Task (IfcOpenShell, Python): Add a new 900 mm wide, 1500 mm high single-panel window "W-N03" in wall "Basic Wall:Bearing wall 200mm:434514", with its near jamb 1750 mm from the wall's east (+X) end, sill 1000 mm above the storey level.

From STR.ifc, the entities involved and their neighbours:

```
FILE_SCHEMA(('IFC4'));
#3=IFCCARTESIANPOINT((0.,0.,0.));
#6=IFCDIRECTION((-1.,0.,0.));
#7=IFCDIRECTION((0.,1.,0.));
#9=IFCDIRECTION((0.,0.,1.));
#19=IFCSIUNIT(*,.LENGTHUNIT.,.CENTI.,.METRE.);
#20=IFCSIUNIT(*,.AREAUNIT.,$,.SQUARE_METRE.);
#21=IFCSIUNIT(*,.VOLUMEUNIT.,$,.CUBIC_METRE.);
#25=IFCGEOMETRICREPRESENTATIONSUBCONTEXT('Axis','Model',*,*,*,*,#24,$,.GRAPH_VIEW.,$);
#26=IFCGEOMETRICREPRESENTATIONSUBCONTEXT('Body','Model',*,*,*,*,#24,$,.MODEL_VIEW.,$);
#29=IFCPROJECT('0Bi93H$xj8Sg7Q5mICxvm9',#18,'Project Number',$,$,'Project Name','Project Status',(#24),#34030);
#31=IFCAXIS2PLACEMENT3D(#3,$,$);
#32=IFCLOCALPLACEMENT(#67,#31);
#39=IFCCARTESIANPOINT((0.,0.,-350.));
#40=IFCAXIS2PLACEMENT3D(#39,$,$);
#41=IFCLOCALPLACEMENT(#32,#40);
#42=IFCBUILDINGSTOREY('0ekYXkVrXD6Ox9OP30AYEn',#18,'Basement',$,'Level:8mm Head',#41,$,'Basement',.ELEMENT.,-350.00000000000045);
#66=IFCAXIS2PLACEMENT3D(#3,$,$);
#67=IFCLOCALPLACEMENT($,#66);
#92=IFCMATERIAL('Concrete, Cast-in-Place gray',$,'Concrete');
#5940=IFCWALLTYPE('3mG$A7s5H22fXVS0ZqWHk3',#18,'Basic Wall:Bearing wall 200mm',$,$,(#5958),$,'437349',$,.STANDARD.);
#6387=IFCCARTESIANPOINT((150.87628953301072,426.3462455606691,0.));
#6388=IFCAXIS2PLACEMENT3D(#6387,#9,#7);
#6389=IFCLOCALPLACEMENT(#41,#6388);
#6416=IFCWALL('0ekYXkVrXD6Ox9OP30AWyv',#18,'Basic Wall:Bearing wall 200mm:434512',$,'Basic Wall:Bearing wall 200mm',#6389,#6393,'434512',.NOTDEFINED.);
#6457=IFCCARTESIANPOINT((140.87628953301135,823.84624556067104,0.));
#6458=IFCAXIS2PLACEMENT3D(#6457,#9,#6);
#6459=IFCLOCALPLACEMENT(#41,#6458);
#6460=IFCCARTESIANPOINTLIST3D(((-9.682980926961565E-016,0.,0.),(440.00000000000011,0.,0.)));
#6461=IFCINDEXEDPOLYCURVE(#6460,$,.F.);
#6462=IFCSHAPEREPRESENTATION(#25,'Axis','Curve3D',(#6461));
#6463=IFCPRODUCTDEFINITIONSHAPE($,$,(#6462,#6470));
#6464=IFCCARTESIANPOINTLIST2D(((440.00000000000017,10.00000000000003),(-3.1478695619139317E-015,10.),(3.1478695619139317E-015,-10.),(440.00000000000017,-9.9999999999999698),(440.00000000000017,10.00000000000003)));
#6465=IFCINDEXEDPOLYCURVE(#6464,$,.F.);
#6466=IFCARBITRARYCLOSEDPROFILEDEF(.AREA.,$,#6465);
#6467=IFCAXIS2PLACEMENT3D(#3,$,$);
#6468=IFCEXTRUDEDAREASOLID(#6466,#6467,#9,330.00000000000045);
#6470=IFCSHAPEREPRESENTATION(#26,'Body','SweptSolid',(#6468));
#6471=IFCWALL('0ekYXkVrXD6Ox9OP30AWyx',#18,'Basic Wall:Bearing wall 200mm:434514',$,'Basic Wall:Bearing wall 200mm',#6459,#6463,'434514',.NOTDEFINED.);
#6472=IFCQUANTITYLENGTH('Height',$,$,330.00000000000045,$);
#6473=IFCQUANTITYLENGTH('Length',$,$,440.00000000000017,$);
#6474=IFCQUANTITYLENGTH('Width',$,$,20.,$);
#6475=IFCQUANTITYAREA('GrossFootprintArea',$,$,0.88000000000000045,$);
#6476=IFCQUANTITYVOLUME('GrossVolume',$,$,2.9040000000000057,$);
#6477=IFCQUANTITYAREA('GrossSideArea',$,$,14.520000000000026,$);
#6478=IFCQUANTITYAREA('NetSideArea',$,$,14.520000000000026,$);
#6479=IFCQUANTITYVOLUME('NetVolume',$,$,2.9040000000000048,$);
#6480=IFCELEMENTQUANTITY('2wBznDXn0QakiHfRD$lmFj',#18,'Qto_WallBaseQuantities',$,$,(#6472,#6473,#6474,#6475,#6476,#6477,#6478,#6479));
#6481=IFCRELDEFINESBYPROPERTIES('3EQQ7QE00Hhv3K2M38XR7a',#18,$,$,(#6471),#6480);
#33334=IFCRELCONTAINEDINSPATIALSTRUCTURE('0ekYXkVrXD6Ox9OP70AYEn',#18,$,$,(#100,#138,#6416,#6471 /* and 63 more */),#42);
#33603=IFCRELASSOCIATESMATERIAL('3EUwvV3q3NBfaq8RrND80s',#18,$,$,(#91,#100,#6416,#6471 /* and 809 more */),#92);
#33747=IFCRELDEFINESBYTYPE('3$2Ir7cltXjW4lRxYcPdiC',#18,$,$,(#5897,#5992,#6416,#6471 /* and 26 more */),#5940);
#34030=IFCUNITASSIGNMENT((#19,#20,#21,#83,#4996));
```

```python
import numpy as np
import ifcopenshell
import ifcopenshell.api.feature
import ifcopenshell.api.geometry
import ifcopenshell.api.pset
import ifcopenshell.api.root
import ifcopenshell.api.spatial
import ifcopenshell.geom
import ifcopenshell.util.element
import ifcopenshell.util.placement
import ifcopenshell.util.representation
import ifcopenshell.util.shape
import ifcopenshell.util.unit

model = ifcopenshell.open("STR.ifc")
unit_scale = ifcopenshell.util.unit.calculate_unit_scale(model)
area_scale = ifcopenshell.util.unit.calculate_unit_scale(model, "AREAUNIT")
volume_scale = ifcopenshell.util.unit.calculate_unit_scale(model, "VOLUMEUNIT")
settings = ifcopenshell.geom.settings()


def volume(element):
    """Net volume in cubic metres, openings subtracted."""
    shape = ifcopenshell.geom.create_shape(settings, element)
    return ifcopenshell.util.shape.get_volume(shape.geometry)


wall = model.by_guid("0ekYXkVrXD6Ox9OP30AWyx")
storey = ifcopenshell.util.element.get_container(wall, ifc_class="IfcBuildingStorey")
context = ifcopenshell.util.representation.get_context(model, "Model", "Body", "MODEL_VIEW")
before = volume(wall)

width, height, from_end, sill = 0.9, 1.5, 1.75, 1  # metres

# The wall runs along its own X axis, and the end named is its -X end.
wall_shape = ifcopenshell.geom.create_shape(settings, wall)
x, y, z = ifcopenshell.util.shape.get_vertices(wall_shape.geometry).T
start = x.min() + from_end
face, thickness = float(y.min()), float(y.max() - y.min())
wall_matrix = ifcopenshell.util.placement.get_local_placement(wall.ObjectPlacement)
level = ifcopenshell.util.placement.get_local_placement(storey.ObjectPlacement)[2, 3]


def in_wall(x, y):
    """Placement at x, y metres in the wall's axes, at sill height."""
    matrix = wall_matrix.copy()
    matrix[:, 3] = wall_matrix @ np.array([x / unit_scale, y / unit_scale, 0.0, 1.0])
    matrix[2, 3] = level + sill / unit_scale
    return matrix


# Opening: a box that overshoots both wall faces by 50 mm.
opening = ifcopenshell.api.root.create_entity(model, ifc_class="IfcOpeningElement", predefined_type="OPENING")
box = ifcopenshell.api.geometry.add_wall_representation(
    model, context=context, length=width, height=height, thickness=thickness + 0.1
)
ifcopenshell.api.geometry.assign_representation(model, product=opening, representation=box)
ifcopenshell.api.geometry.edit_object_placement(model, product=opening, matrix=in_wall(start, face - 0.05), is_si=False)
ifcopenshell.api.feature.add_feature(model, feature=opening, element=wall)

window = ifcopenshell.api.root.create_entity(model, ifc_class="IfcWindow", name="W-N03", predefined_type="WINDOW")
window.OverallWidth, window.OverallHeight = width / unit_scale, height / unit_scale
window.PartitioningType = "SINGLE_PANEL"
body = ifcopenshell.api.geometry.add_window_representation(
    model,
    context=context,
    overall_width=window.OverallWidth,
    overall_height=window.OverallHeight,
    partition_type="SINGLE_PANEL",
)
ifcopenshell.api.geometry.assign_representation(model, product=window, representation=body)
ifcopenshell.api.spatial.assign_container(model, products=[window], relating_structure=storey)
ifcopenshell.api.feature.add_filling(model, opening=opening, element=window)

# Centre the window in the wall's thickness.
ifcopenshell.api.geometry.edit_object_placement(model, product=window, matrix=in_wall(start, face), is_si=False)
window_shape = ifcopenshell.geom.create_shape(settings, window)
depth = ifcopenshell.util.shape.get_vertices(window_shape.geometry)[:, 1]
offset = face + thickness / 2 - (depth.min() + depth.max()) / 2
ifcopenshell.api.geometry.edit_object_placement(model, product=window, matrix=in_wall(start, offset), is_si=False)

after = volume(wall)

# Update the wall's stored quantities.
qto = model.by_id(ifcopenshell.util.element.get_pset(wall, "Qto_WallBaseQuantities", should_inherit=False)["id"])
ifcopenshell.api.pset.edit_qto(model, qto=qto, properties={
    "NetSideArea": after / thickness / area_scale,
    "NetVolume": after / volume_scale,
})

print(f"wall volume {before:.3f} -> {after:.3f} m3")

model.write("STR_edited.ifc")
```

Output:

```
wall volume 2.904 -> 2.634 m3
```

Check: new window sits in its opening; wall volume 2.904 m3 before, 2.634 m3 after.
